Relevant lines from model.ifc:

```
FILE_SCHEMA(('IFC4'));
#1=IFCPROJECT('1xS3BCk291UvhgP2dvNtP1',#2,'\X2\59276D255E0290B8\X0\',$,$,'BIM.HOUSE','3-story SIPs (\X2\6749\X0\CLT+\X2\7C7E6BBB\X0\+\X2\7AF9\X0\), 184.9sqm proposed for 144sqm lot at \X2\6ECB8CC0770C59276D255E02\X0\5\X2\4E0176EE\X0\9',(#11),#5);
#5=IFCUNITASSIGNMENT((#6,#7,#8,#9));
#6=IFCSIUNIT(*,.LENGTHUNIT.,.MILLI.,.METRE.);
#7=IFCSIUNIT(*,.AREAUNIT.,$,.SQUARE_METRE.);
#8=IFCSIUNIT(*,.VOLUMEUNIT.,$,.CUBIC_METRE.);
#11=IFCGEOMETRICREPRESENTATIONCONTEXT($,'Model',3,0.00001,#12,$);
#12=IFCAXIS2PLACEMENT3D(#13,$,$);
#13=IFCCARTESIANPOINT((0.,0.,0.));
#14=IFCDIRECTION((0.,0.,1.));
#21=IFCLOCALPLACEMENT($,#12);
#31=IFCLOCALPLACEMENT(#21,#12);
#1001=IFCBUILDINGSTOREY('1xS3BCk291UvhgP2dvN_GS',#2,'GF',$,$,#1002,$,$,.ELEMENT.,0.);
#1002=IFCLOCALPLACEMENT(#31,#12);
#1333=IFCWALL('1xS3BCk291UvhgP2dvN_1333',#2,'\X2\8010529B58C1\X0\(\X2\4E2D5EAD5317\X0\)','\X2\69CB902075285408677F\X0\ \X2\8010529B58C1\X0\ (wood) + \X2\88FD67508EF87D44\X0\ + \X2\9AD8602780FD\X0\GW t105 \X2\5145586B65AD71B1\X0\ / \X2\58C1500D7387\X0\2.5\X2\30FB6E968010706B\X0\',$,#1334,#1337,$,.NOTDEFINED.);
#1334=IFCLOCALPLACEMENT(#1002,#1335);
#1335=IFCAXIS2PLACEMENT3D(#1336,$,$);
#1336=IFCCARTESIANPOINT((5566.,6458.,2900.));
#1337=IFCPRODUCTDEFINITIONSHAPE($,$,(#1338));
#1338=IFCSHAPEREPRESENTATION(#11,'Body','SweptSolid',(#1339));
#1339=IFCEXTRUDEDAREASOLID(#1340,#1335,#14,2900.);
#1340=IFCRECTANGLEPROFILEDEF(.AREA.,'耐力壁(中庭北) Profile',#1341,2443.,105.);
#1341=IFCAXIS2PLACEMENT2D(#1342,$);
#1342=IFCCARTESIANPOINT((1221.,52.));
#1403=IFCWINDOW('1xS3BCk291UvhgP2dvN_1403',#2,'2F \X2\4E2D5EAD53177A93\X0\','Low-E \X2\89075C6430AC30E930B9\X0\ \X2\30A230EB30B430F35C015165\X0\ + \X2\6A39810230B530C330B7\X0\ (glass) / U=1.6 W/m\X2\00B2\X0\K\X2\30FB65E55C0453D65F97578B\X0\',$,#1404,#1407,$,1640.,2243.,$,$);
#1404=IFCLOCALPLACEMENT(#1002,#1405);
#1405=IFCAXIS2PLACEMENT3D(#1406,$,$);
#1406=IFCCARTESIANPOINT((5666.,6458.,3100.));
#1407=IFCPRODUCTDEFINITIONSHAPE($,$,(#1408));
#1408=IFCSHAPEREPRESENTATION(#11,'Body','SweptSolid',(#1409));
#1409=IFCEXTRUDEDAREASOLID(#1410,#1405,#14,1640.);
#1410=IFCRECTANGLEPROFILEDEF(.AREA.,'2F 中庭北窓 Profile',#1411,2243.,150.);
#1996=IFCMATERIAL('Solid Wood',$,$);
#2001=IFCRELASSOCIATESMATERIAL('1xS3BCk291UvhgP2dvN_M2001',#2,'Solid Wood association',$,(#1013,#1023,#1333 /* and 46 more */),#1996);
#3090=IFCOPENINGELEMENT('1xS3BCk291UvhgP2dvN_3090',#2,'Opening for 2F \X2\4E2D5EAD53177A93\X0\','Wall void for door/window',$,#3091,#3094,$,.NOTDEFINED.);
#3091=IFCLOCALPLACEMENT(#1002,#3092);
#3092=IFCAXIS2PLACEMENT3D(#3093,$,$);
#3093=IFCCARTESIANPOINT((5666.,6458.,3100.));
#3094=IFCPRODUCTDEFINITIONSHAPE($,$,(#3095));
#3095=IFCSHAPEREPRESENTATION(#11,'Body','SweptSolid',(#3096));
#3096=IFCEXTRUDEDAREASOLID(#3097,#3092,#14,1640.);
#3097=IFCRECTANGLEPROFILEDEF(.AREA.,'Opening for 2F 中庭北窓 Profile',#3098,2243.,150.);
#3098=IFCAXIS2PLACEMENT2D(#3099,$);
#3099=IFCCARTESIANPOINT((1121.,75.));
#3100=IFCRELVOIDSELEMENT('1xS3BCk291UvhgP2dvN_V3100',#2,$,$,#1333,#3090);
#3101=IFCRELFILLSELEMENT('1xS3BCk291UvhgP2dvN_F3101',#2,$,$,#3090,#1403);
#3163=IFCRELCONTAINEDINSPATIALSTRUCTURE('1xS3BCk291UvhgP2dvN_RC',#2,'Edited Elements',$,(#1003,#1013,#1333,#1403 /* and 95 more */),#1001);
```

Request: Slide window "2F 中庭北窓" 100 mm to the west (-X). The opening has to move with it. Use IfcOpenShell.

```python
import ifcopenshell
import ifcopenshell.api.geometry
import ifcopenshell.util.placement
import ifcopenshell.util.unit

model = ifcopenshell.open("model.ifc")
unit_scale = ifcopenshell.util.unit.calculate_unit_scale(model)

window = model.by_guid("1xS3BCk291UvhgP2dvN_1403")
opening = window.FillsVoids[0].RelatingOpeningElement
wall = opening.VoidsElements[0].RelatingBuildingElement

wall_matrix = ifcopenshell.util.placement.get_local_placement(wall.ObjectPlacement)
shift = wall_matrix[:3, 0] * -0.1 / unit_scale
before = ifcopenshell.util.placement.get_local_placement(window.ObjectPlacement)[:3, 3].copy()

# The window is not placed relative to its opening, so move both.
for product in (opening, window):
    matrix = ifcopenshell.util.placement.get_local_placement(product.ObjectPlacement)
    matrix[:3, 3] += shift
    ifcopenshell.api.geometry.edit_object_placement(model, product=product, matrix=matrix, is_si=False)

after = ifcopenshell.util.placement.get_local_placement(window.ObjectPlacement)[:3, 3]
print("window moved by", (after - before).round(3) + 0.0)

model.write("model_rev.ifc")
```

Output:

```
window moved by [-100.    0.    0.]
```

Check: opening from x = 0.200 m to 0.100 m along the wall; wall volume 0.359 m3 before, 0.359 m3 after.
